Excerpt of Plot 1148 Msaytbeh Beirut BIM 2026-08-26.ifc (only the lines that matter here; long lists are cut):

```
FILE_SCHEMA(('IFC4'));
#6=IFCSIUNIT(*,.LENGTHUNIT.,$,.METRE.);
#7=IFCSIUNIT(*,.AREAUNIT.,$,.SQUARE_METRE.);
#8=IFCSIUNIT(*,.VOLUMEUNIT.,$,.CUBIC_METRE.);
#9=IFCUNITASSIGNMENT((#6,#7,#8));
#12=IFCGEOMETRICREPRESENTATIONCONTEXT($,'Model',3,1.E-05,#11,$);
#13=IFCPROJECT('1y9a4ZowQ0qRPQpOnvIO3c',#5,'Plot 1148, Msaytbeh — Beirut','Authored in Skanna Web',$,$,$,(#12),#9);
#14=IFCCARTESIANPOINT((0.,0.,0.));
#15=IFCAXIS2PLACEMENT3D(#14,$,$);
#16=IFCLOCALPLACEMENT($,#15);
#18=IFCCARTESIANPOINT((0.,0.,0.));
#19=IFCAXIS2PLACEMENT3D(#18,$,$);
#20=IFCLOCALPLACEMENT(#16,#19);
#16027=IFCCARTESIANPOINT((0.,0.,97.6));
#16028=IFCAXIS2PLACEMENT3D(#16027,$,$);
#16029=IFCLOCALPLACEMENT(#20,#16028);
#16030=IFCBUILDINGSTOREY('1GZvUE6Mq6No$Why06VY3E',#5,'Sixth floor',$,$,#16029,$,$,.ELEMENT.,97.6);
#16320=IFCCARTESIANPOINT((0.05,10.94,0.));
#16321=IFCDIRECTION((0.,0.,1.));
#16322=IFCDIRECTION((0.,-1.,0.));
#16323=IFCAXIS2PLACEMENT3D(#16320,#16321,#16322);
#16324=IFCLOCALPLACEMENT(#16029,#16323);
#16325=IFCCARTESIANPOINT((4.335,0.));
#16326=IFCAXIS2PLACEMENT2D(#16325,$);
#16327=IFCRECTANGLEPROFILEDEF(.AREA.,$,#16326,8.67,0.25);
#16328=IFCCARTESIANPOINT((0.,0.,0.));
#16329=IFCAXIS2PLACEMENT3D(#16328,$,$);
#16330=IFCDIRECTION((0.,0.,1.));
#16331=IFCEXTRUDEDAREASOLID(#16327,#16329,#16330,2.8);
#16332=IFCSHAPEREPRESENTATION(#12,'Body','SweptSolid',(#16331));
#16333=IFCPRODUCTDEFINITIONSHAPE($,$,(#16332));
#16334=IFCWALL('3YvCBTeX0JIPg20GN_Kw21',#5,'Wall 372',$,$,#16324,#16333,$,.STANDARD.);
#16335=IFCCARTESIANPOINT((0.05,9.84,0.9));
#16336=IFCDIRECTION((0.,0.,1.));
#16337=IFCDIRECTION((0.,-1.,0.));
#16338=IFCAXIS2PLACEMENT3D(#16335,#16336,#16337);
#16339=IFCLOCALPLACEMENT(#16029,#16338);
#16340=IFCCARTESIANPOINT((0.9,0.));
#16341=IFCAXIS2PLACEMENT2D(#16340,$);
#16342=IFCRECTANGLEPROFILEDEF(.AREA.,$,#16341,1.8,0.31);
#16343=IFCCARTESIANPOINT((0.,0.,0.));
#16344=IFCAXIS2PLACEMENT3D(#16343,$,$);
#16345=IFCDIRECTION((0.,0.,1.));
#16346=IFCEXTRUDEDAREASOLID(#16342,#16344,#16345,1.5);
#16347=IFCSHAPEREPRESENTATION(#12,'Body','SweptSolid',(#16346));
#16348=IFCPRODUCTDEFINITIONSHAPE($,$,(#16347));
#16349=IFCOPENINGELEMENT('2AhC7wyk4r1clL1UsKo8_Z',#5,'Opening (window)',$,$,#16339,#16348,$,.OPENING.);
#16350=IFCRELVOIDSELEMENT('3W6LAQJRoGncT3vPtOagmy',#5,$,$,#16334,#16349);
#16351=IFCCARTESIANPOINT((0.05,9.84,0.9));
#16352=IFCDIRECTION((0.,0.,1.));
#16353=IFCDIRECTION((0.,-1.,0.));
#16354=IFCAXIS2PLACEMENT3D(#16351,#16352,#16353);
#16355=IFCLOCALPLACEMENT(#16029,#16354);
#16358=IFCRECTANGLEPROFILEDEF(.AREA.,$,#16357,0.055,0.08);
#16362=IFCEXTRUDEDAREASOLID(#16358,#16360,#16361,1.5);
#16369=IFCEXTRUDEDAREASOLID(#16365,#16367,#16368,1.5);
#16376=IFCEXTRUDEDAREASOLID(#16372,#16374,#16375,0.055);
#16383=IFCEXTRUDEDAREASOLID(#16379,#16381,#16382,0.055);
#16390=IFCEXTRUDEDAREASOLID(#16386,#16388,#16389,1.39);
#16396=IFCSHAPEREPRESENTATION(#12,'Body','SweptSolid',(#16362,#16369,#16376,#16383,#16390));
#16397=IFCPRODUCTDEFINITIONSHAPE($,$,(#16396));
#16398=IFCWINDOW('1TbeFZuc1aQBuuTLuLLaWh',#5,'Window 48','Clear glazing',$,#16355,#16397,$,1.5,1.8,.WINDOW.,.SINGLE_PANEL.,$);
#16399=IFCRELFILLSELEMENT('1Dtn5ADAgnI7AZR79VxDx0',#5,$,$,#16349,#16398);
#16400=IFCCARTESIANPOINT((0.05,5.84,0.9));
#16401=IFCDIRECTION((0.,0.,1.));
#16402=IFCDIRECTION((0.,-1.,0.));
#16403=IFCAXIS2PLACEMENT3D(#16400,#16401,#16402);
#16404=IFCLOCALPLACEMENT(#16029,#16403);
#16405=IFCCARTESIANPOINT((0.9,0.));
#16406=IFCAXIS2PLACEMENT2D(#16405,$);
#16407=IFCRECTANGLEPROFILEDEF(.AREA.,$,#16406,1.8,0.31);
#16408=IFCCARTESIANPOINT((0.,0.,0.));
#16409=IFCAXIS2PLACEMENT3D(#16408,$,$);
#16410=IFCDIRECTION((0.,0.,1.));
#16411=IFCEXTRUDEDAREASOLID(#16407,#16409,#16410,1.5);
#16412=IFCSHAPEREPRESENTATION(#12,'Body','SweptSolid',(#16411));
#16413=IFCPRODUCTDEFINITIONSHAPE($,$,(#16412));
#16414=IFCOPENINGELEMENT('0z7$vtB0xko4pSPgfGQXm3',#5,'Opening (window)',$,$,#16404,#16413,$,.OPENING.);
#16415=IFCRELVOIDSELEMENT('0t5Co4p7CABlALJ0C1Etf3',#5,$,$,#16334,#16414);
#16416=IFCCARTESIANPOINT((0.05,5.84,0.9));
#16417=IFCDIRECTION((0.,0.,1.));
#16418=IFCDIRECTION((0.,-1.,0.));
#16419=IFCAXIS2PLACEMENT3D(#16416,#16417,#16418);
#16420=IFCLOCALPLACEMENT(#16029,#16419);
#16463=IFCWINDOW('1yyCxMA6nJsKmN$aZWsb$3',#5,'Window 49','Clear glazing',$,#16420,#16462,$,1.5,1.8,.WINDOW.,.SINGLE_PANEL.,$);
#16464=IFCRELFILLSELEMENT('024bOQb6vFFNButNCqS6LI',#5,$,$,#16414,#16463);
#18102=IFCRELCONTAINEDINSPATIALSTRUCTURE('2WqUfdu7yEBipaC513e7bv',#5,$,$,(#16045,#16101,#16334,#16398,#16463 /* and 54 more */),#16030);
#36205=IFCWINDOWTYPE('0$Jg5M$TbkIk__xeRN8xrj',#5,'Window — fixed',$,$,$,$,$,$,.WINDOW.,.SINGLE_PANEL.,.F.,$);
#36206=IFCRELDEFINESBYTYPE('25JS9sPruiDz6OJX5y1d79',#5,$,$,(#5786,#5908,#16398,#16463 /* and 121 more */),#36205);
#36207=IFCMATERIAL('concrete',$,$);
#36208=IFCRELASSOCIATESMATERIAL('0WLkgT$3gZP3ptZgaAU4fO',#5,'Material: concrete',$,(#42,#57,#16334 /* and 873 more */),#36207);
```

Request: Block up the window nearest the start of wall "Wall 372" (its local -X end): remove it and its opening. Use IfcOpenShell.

```python
import ifcopenshell
import ifcopenshell.api.feature
import ifcopenshell.api.root
import ifcopenshell.geom
import ifcopenshell.util.shape

model = ifcopenshell.open("Plot 1148 Msaytbeh Beirut BIM 2026-08-26.ifc")
settings = ifcopenshell.geom.settings()


def volume(element):
    """Net volume in cubic metres, openings subtracted."""
    shape = ifcopenshell.geom.create_shape(settings, element)
    return ifcopenshell.util.shape.get_volume(shape.geometry)


window = model.by_guid("1TbeFZuc1aQBuuTLuLLaWh")
opening = window.FillsVoids[0].RelatingOpeningElement
wall = opening.VoidsElements[0].RelatingBuildingElement
before = volume(wall)

ifcopenshell.api.root.remove_product(model, product=window)
ifcopenshell.api.feature.remove_feature(model, feature=opening)

after = volume(wall)

print(f"wall volume {before:.3f} -> {after:.3f} m3")

model.write("Plot 1148 Msaytbeh Beirut BIM 2026-08-26_updated.ifc")
```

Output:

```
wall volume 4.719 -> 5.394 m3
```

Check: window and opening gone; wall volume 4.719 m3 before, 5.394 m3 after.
